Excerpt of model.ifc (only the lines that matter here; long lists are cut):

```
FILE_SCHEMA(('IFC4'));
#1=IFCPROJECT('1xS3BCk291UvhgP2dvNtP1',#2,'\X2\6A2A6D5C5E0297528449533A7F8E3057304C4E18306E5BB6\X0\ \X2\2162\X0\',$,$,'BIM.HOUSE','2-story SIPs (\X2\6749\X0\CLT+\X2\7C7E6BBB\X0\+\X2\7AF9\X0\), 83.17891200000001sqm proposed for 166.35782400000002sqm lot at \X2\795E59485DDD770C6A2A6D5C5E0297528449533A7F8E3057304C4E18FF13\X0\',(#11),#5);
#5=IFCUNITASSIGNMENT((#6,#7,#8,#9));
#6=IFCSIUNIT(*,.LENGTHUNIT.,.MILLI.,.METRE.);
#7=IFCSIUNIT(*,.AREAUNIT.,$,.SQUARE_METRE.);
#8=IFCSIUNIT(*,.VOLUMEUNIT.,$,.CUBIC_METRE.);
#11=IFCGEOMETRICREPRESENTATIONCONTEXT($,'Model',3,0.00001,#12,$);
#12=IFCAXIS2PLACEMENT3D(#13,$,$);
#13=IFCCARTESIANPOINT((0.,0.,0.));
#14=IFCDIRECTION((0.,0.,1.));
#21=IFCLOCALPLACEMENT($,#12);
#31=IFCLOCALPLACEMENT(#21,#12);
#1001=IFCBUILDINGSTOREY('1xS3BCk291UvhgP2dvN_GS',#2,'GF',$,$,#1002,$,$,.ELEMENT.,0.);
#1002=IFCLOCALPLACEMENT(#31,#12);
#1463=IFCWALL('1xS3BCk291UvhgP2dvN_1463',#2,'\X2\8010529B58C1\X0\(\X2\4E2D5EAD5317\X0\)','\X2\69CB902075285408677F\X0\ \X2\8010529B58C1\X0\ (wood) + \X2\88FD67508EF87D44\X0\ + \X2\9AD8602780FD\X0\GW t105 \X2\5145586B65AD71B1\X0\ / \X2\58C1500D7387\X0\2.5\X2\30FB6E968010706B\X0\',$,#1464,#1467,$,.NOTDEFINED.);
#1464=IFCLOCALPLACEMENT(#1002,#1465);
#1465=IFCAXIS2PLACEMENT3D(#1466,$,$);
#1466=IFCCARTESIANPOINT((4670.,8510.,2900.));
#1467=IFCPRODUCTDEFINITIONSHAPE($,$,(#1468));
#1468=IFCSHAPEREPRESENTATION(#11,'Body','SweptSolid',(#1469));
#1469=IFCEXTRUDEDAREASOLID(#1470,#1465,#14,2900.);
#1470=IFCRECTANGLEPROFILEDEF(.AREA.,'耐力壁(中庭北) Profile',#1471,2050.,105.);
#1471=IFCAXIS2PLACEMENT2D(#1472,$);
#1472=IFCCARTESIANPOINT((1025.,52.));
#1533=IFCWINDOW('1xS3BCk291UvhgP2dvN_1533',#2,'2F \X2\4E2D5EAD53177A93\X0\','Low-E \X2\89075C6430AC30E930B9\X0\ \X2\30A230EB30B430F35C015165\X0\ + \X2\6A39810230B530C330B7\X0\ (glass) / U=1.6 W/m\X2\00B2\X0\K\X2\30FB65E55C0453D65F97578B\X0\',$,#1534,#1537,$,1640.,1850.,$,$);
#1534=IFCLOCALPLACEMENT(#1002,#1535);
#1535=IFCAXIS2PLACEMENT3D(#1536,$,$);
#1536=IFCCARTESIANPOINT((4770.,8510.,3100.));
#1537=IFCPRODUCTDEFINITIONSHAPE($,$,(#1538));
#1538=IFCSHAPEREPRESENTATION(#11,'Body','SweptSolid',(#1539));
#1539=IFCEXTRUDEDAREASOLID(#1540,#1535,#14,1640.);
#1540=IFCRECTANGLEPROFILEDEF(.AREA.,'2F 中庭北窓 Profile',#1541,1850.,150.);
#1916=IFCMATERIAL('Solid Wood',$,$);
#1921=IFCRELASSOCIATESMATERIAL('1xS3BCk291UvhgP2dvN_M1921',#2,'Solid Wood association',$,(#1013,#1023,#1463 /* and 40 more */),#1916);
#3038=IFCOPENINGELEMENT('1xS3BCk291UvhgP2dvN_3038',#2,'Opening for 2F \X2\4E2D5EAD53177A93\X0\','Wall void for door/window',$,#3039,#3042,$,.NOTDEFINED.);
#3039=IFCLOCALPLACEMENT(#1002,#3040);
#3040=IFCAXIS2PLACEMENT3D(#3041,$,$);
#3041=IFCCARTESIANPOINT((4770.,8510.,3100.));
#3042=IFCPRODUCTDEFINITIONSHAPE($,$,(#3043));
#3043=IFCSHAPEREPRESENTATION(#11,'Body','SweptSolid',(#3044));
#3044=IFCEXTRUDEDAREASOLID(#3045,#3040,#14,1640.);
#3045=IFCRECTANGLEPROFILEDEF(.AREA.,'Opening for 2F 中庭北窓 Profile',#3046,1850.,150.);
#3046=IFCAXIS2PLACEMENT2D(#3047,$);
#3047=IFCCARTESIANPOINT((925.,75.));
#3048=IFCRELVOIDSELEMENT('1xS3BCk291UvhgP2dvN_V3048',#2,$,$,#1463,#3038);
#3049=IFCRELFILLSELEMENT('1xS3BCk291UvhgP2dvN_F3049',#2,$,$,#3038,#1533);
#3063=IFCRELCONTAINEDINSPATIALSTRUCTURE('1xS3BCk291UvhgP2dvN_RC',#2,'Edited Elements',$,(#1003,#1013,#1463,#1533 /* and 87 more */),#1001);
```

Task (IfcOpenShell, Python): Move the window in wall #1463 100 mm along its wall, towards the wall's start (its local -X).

```python
import ifcopenshell
import ifcopenshell.api.geometry
import ifcopenshell.util.placement
import ifcopenshell.util.unit

model = ifcopenshell.open("model.ifc")
unit_scale = ifcopenshell.util.unit.calculate_unit_scale(model)

window = model.by_id(1533)
opening = window.FillsVoids[0].RelatingOpeningElement
wall = opening.VoidsElements[0].RelatingBuildingElement

wall_matrix = ifcopenshell.util.placement.get_local_placement(wall.ObjectPlacement)
shift = wall_matrix[:3, 0] * -0.1 / unit_scale
before = ifcopenshell.util.placement.get_local_placement(window.ObjectPlacement)[:3, 3].copy()

# The window is not placed relative to its opening, so move both.
for product in (opening, window):
    matrix = ifcopenshell.util.placement.get_local_placement(product.ObjectPlacement)
    matrix[:3, 3] += shift
    ifcopenshell.api.geometry.edit_object_placement(model, product=product, matrix=matrix, is_si=False)

after = ifcopenshell.util.placement.get_local_placement(window.ObjectPlacement)[:3, 3]
print("window moved by", (after - before).round(3) + 0.0)

model.write("model-out.ifc")
```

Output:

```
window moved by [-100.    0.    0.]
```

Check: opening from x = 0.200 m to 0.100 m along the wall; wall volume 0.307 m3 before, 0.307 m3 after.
